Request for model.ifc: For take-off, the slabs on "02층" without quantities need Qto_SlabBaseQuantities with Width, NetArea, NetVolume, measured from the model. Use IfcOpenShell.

First a look at what the model holds.

```python
import ifcopenshell
import ifcopenshell.util.element
import ifcopenshell.util.unit

model = ifcopenshell.open("model.ifc")
print(model.schema)
for unit_type in ("LENGTHUNIT", "AREAUNIT", "VOLUMEUNIT"):
    print(unit_type, ifcopenshell.util.unit.calculate_unit_scale(model, unit_type))
storey = next(s for s in model.by_type("IfcBuildingStorey") if s.Name == "02층")
slabs = [e for e in ifcopenshell.util.element.get_decomposition(storey) if e.is_a("IfcSlab")]
for e in sorted(slabs, key=lambda e: e.id()):
    print(e.id(), e.is_a(), e.Name, list(ifcopenshell.util.element.get_psets(e, qtos_only=True)), sep=" | ")
```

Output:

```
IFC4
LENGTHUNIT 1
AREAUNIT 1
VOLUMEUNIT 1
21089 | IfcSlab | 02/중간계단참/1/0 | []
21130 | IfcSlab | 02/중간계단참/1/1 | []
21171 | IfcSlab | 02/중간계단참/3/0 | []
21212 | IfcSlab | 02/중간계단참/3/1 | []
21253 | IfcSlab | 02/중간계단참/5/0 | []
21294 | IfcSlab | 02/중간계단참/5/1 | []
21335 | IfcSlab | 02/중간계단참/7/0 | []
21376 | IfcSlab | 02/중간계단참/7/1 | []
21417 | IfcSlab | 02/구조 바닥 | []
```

```python
import ifcopenshell
import ifcopenshell.api.pset
import ifcopenshell.geom
import ifcopenshell.util.element
import ifcopenshell.util.shape
import ifcopenshell.util.unit

model = ifcopenshell.open("model.ifc")
unit_scale = ifcopenshell.util.unit.calculate_unit_scale(model)
area_scale = ifcopenshell.util.unit.calculate_unit_scale(model, "AREAUNIT")
volume_scale = ifcopenshell.util.unit.calculate_unit_scale(model, "VOLUMEUNIT")
settings = ifcopenshell.geom.settings()

storey = next(s for s in model.by_type("IfcBuildingStorey") if s.Name == "02층")
slabs = [e for e in ifcopenshell.util.element.get_decomposition(storey) if e.is_a("IfcSlab")]

for e in sorted(slabs, key=lambda e: e.id()):
    if ifcopenshell.util.element.get_psets(e, qtos_only=True, should_inherit=False):
        continue
    # Geometry comes back in metres, in the element's own axes.
    shape = ifcopenshell.geom.create_shape(settings, e)
    values = {
        "Width": ifcopenshell.util.shape.get_z(shape.geometry) / unit_scale,
        "NetArea": ifcopenshell.util.shape.get_footprint_area(shape.geometry) / area_scale,
        "NetVolume": ifcopenshell.util.shape.get_volume(shape.geometry) / volume_scale,
    }
    qto = ifcopenshell.api.pset.add_qto(model, product=e, name="Qto_SlabBaseQuantities")
    ifcopenshell.api.pset.edit_qto(model, qto=qto, properties=values)
    print(e.id(), {k: round(v, 3) for k, v in values.items()})

model.write("model-out.ifc")
```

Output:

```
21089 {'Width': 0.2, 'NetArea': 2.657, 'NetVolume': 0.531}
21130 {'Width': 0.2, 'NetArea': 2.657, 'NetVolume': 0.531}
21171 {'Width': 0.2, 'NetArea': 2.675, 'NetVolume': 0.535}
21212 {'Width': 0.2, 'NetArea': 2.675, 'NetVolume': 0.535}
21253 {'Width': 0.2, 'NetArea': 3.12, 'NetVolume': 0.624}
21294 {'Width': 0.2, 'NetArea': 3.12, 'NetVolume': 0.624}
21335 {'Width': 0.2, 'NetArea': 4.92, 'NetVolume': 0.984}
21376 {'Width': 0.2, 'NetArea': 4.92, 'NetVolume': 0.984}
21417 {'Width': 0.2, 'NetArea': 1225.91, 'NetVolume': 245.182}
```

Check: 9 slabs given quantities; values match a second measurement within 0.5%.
